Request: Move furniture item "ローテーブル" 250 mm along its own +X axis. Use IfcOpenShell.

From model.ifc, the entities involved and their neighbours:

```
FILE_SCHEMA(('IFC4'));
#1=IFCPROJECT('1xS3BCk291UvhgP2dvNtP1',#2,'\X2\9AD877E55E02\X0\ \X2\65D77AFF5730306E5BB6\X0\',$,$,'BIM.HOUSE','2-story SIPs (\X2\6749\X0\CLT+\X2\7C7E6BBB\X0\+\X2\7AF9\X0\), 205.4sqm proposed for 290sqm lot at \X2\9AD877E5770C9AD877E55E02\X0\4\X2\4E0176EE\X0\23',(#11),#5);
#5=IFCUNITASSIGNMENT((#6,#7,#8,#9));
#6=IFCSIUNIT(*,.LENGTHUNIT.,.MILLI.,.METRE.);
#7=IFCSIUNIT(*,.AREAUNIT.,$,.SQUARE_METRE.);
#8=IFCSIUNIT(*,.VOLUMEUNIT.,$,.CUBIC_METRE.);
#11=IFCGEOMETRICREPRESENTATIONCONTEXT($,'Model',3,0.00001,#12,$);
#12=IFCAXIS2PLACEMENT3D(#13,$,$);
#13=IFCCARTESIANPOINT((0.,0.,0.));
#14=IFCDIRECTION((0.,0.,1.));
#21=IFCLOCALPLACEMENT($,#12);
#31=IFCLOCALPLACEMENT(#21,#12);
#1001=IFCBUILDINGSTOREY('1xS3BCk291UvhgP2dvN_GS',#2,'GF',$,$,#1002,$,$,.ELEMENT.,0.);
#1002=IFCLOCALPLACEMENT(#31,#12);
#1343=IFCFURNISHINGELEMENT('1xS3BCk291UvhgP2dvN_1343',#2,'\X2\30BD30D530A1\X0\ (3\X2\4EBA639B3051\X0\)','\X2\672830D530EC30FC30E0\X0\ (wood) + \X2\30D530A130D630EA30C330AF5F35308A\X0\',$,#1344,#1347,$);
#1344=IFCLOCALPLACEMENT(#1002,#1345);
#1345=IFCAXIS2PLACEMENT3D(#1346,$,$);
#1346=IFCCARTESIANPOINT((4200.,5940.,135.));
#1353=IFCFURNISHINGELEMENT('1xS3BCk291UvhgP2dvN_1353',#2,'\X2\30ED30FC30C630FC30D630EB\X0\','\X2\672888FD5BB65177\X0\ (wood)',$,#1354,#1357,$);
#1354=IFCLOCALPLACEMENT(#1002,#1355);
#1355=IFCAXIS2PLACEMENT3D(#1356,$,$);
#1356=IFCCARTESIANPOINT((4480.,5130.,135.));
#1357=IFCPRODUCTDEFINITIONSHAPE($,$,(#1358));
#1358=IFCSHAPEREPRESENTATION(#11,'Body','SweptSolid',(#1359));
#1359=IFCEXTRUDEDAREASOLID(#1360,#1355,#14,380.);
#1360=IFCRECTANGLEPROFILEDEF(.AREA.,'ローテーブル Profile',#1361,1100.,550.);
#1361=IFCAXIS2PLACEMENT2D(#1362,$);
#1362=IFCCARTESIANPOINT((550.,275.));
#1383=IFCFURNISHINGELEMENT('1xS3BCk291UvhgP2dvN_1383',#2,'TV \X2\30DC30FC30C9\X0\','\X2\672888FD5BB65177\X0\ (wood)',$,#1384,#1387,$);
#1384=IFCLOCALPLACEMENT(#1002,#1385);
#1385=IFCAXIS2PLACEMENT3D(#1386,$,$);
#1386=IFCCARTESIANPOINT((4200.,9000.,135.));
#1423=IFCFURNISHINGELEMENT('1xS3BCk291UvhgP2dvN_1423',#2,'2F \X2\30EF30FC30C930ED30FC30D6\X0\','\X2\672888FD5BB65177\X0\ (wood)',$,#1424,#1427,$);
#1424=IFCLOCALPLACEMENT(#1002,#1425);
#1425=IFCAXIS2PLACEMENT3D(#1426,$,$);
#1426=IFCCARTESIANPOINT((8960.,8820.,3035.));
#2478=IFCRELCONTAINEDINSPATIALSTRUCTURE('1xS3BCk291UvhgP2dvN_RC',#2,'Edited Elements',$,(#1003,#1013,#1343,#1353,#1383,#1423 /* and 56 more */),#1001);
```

```python
import ifcopenshell
import ifcopenshell.api.geometry
import ifcopenshell.util.placement

model = ifcopenshell.open("model.ifc")

item = model.by_guid("1xS3BCk291UvhgP2dvN_1353")
matrix = ifcopenshell.util.placement.get_local_placement(item.ObjectPlacement)
matrix[:3, 3] += matrix[:3, 0] * 250.0
ifcopenshell.api.geometry.edit_object_placement(model, product=item, matrix=matrix, is_si=False)

print(ifcopenshell.util.placement.get_local_placement(item.ObjectPlacement).round(3) + 0.0)

model.write("model_updated.ifc")
```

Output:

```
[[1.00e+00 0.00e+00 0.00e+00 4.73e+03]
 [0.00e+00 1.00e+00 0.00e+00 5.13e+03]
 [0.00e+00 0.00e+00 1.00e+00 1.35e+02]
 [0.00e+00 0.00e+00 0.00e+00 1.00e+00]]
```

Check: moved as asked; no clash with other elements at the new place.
